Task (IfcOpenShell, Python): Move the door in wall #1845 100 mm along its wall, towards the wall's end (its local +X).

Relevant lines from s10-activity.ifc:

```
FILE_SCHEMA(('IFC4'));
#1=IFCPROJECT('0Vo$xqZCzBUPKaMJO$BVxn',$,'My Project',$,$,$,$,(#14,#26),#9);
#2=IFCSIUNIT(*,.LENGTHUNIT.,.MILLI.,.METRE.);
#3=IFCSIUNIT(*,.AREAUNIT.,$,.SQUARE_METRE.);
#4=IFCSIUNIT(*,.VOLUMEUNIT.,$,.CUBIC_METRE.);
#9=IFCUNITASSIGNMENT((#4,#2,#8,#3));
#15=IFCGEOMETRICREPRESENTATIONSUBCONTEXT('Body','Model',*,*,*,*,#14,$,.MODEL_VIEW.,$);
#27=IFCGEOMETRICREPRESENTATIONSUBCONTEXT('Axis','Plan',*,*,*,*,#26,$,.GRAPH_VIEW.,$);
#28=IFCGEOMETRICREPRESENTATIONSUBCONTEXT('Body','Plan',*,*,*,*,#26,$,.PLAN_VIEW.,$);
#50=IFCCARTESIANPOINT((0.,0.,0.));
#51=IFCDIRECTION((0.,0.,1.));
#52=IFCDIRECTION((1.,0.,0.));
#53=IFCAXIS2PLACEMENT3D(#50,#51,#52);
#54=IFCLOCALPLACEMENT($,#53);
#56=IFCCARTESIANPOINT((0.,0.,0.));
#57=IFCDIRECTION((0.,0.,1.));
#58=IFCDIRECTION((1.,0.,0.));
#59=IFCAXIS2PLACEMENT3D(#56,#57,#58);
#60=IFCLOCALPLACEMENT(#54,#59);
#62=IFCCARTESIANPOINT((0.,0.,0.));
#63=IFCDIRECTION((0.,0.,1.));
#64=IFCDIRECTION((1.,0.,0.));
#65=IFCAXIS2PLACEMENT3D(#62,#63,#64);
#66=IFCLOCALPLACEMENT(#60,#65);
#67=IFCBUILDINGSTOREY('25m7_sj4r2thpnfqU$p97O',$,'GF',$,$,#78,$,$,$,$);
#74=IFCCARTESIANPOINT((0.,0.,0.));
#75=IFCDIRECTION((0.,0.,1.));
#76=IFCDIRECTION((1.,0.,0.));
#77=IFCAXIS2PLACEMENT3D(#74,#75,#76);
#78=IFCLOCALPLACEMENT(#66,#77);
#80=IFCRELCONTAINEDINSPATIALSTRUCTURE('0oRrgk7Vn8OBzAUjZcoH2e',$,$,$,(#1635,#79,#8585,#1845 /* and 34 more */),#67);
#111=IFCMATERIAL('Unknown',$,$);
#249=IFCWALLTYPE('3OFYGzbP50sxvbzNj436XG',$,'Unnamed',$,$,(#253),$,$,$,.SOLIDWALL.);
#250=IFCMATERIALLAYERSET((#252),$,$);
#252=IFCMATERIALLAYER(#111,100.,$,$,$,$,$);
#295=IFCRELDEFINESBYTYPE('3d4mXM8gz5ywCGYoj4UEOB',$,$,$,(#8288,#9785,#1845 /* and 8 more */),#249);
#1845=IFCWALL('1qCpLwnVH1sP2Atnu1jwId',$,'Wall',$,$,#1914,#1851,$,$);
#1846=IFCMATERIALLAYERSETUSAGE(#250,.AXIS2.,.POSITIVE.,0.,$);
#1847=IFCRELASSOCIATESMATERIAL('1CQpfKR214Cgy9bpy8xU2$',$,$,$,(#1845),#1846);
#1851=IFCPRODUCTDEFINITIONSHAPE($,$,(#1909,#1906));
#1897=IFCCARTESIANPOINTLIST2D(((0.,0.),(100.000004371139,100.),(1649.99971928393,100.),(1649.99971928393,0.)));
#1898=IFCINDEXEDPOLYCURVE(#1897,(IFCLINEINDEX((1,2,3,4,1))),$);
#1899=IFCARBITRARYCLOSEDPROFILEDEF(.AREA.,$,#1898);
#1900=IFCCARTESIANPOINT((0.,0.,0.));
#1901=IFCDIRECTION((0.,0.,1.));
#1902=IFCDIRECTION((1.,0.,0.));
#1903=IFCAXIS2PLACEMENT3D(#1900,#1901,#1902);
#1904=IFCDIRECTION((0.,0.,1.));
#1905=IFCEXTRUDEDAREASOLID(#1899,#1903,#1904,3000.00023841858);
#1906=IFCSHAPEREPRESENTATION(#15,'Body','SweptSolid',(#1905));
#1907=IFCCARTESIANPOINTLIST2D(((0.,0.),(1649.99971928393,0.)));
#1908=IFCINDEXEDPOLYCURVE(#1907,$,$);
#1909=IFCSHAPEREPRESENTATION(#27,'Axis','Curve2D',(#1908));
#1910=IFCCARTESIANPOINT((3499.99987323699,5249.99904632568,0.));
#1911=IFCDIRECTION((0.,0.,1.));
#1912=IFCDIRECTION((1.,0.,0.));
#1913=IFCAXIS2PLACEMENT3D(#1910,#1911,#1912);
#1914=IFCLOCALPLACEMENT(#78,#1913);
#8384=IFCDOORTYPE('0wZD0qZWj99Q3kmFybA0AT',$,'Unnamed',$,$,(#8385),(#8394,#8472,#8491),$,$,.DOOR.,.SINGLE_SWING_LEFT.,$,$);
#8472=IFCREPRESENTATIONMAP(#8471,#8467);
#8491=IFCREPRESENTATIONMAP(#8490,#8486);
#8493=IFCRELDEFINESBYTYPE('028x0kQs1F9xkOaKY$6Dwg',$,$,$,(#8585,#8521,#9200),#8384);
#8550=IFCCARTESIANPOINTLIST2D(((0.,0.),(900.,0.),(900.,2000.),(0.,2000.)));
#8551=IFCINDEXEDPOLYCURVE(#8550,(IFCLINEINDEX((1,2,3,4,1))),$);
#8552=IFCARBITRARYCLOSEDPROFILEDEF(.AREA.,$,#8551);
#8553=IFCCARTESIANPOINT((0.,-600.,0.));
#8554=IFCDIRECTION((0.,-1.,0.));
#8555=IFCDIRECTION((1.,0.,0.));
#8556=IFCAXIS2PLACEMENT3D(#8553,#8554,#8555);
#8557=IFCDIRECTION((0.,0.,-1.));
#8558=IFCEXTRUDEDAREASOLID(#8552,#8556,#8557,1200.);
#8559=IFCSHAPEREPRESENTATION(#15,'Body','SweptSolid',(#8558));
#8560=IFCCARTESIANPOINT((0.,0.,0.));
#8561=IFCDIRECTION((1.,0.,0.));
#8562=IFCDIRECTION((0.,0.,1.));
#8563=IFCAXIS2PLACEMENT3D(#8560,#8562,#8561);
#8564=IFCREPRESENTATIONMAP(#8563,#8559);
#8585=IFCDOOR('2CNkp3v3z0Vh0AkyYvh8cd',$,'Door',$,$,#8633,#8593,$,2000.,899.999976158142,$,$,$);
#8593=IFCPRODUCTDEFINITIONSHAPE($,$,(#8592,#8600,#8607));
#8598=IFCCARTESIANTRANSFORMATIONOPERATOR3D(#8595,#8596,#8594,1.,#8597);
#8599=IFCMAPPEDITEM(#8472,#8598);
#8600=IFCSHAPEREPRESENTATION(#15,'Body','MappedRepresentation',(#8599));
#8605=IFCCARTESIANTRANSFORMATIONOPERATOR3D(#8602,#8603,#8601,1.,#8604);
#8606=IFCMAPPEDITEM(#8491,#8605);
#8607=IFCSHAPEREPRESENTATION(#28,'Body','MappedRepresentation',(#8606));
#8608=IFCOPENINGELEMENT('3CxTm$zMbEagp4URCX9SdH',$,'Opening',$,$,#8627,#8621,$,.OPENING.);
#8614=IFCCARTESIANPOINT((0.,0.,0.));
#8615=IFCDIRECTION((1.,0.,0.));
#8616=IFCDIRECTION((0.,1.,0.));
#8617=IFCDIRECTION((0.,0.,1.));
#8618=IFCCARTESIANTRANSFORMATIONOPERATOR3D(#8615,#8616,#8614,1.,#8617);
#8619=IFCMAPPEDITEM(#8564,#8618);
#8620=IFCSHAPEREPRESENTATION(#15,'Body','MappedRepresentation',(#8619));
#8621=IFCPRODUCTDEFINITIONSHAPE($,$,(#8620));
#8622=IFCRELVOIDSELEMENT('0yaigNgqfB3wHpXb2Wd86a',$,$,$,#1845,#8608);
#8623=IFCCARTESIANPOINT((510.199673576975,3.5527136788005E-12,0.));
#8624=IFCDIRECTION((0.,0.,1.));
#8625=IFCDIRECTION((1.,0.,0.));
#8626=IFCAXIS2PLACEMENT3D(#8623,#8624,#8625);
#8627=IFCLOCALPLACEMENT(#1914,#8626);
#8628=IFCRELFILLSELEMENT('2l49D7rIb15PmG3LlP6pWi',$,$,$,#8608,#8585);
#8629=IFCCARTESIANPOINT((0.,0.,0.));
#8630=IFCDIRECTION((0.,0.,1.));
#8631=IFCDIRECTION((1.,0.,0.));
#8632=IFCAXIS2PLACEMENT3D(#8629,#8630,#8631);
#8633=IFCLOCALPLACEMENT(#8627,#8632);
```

```python
import ifcopenshell
import ifcopenshell.api.geometry
import ifcopenshell.util.placement
import ifcopenshell.util.unit

model = ifcopenshell.open("s10-activity.ifc")
unit_scale = ifcopenshell.util.unit.calculate_unit_scale(model)

door = model.by_guid("2CNkp3v3z0Vh0AkyYvh8cd")
opening = door.FillsVoids[0].RelatingOpeningElement
wall = opening.VoidsElements[0].RelatingBuildingElement

wall_matrix = ifcopenshell.util.placement.get_local_placement(wall.ObjectPlacement)
shift = wall_matrix[:3, 0] * 0.1 / unit_scale
before = ifcopenshell.util.placement.get_local_placement(door.ObjectPlacement)[:3, 3].copy()

# The door is placed relative to its opening, so it follows when the opening moves.
matrix = ifcopenshell.util.placement.get_local_placement(opening.ObjectPlacement)
matrix[:3, 3] += shift
ifcopenshell.api.geometry.edit_object_placement(
    model, product=opening, matrix=matrix, is_si=False, should_transform_children=True
)

after = ifcopenshell.util.placement.get_local_placement(door.ObjectPlacement)[:3, 3]
print("door moved by", (after - before).round(3) + 0.0)

model.write("s10-activity_rev.ifc")
```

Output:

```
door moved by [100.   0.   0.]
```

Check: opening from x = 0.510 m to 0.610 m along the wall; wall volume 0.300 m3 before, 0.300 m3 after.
